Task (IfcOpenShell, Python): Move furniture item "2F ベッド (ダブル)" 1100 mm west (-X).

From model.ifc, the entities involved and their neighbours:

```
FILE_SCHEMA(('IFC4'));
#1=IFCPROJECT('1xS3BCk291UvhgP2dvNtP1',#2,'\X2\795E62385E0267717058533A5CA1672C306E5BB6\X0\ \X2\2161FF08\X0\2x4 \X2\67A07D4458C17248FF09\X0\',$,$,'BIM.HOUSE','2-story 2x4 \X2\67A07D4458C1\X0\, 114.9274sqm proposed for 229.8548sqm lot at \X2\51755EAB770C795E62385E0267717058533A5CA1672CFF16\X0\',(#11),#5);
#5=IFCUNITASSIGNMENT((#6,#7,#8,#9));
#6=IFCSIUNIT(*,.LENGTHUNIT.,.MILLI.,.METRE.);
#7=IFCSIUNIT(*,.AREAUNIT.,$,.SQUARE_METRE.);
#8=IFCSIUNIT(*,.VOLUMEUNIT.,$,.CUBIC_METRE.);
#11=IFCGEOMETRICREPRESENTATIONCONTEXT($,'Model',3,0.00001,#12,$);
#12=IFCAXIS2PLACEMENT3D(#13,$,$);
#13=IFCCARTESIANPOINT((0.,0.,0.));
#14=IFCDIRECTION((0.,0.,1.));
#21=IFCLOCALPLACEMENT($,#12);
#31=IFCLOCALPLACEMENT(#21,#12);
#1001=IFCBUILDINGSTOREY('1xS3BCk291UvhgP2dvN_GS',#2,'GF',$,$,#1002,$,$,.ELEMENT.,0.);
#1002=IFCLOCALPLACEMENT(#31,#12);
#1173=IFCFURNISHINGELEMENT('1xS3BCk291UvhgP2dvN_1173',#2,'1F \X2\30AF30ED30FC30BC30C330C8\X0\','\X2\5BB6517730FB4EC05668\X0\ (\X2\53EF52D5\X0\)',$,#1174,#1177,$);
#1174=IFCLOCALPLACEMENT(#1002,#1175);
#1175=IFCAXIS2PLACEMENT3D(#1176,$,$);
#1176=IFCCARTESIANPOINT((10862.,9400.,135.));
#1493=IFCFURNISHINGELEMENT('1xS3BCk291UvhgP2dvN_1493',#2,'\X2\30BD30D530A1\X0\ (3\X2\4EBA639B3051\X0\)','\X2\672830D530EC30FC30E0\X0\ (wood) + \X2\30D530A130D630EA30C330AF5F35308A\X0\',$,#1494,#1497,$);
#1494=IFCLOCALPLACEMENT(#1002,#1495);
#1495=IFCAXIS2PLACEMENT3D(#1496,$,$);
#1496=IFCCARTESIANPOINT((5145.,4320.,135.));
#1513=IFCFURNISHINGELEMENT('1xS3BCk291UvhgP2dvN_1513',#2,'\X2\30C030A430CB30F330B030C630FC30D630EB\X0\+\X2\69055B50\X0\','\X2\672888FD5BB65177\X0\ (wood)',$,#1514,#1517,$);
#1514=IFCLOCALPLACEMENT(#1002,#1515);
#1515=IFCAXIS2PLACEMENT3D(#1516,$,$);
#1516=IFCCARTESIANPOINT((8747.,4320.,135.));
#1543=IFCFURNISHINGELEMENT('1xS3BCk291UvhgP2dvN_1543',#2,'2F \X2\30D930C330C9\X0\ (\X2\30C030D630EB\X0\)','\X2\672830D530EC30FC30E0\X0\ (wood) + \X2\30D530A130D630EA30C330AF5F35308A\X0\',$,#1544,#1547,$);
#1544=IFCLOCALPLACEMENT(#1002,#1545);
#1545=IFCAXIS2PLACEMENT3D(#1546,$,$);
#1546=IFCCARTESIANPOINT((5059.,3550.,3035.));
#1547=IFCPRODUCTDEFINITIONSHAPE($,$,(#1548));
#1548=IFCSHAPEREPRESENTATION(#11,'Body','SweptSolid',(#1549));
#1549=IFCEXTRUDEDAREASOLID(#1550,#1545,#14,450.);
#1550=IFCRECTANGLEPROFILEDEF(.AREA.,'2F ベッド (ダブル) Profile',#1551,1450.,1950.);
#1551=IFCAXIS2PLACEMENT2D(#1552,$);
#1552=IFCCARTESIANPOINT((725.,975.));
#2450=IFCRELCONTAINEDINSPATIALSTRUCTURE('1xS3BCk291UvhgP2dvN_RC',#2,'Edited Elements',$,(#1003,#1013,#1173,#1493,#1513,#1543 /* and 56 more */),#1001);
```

```python
import ifcopenshell
import ifcopenshell.api.geometry
import ifcopenshell.util.placement
import ifcopenshell.util.unit

model = ifcopenshell.open("model.ifc")
unit_scale = ifcopenshell.util.unit.calculate_unit_scale(model)

item = model.by_id(1543)
matrix = ifcopenshell.util.placement.get_local_placement(item.ObjectPlacement)
matrix[0, 3] -= 1.1 / unit_scale
ifcopenshell.api.geometry.edit_object_placement(model, product=item, matrix=matrix, is_si=False)

print(ifcopenshell.util.placement.get_local_placement(item.ObjectPlacement).round(3) + 0.0)

model.write("model_v2.ifc")
```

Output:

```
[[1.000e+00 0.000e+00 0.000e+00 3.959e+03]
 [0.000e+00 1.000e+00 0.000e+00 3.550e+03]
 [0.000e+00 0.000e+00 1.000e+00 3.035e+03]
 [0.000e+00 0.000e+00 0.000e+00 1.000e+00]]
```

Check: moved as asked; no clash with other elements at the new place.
